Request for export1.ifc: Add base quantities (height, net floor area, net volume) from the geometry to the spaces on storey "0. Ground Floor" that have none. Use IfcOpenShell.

First a look at what the model holds.

```python
import ifcopenshell
import ifcopenshell.util.element
import ifcopenshell.util.unit

model = ifcopenshell.open("export1.ifc")
print(model.schema)
for unit_type in ("LENGTHUNIT", "AREAUNIT", "VOLUMEUNIT"):
    print(unit_type, ifcopenshell.util.unit.calculate_unit_scale(model, unit_type))
storey = next(s for s in model.by_type("IfcBuildingStorey") if s.Name == "0. Ground Floor")
spaces = [e for e in ifcopenshell.util.element.get_decomposition(storey) if e.is_a("IfcSpace")]
for e in sorted(spaces, key=lambda e: e.id()):
    print(e.id(), e.is_a(), e.Name, list(ifcopenshell.util.element.get_psets(e, qtos_only=True)), sep=" | ")
```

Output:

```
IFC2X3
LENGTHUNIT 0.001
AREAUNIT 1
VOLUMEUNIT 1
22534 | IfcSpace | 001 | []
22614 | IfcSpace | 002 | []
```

```python
import ifcopenshell
import ifcopenshell.api.pset
import ifcopenshell.geom
import ifcopenshell.util.element
import ifcopenshell.util.shape
import ifcopenshell.util.unit

model = ifcopenshell.open("export1.ifc")
unit_scale = ifcopenshell.util.unit.calculate_unit_scale(model)
area_scale = ifcopenshell.util.unit.calculate_unit_scale(model, "AREAUNIT")
volume_scale = ifcopenshell.util.unit.calculate_unit_scale(model, "VOLUMEUNIT")
settings = ifcopenshell.geom.settings()

storey = next(s for s in model.by_type("IfcBuildingStorey") if s.Name == "0. Ground Floor")
spaces = [e for e in ifcopenshell.util.element.get_decomposition(storey) if e.is_a("IfcSpace")]

for e in sorted(spaces, key=lambda e: e.id()):
    if ifcopenshell.util.element.get_psets(e, qtos_only=True, should_inherit=False):
        continue
    # Geometry comes back in metres, in the element's own axes.
    shape = ifcopenshell.geom.create_shape(settings, e)
    values = {
        "Height": ifcopenshell.util.shape.get_z(shape.geometry) / unit_scale,
        "NetFloorArea": ifcopenshell.util.shape.get_footprint_area(shape.geometry) / area_scale,
        "NetVolume": ifcopenshell.util.shape.get_volume(shape.geometry) / volume_scale,
    }
    qto = ifcopenshell.api.pset.add_qto(model, product=e, name="BaseQuantities")
    ifcopenshell.api.pset.edit_qto(model, qto=qto, properties=values)
    print(e.id(), {k: round(v, 3) for k, v in values.items()})

model.write("export1_updated.ifc")
```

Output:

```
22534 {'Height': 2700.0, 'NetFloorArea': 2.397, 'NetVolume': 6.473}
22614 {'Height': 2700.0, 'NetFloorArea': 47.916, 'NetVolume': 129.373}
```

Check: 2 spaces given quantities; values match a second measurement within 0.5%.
